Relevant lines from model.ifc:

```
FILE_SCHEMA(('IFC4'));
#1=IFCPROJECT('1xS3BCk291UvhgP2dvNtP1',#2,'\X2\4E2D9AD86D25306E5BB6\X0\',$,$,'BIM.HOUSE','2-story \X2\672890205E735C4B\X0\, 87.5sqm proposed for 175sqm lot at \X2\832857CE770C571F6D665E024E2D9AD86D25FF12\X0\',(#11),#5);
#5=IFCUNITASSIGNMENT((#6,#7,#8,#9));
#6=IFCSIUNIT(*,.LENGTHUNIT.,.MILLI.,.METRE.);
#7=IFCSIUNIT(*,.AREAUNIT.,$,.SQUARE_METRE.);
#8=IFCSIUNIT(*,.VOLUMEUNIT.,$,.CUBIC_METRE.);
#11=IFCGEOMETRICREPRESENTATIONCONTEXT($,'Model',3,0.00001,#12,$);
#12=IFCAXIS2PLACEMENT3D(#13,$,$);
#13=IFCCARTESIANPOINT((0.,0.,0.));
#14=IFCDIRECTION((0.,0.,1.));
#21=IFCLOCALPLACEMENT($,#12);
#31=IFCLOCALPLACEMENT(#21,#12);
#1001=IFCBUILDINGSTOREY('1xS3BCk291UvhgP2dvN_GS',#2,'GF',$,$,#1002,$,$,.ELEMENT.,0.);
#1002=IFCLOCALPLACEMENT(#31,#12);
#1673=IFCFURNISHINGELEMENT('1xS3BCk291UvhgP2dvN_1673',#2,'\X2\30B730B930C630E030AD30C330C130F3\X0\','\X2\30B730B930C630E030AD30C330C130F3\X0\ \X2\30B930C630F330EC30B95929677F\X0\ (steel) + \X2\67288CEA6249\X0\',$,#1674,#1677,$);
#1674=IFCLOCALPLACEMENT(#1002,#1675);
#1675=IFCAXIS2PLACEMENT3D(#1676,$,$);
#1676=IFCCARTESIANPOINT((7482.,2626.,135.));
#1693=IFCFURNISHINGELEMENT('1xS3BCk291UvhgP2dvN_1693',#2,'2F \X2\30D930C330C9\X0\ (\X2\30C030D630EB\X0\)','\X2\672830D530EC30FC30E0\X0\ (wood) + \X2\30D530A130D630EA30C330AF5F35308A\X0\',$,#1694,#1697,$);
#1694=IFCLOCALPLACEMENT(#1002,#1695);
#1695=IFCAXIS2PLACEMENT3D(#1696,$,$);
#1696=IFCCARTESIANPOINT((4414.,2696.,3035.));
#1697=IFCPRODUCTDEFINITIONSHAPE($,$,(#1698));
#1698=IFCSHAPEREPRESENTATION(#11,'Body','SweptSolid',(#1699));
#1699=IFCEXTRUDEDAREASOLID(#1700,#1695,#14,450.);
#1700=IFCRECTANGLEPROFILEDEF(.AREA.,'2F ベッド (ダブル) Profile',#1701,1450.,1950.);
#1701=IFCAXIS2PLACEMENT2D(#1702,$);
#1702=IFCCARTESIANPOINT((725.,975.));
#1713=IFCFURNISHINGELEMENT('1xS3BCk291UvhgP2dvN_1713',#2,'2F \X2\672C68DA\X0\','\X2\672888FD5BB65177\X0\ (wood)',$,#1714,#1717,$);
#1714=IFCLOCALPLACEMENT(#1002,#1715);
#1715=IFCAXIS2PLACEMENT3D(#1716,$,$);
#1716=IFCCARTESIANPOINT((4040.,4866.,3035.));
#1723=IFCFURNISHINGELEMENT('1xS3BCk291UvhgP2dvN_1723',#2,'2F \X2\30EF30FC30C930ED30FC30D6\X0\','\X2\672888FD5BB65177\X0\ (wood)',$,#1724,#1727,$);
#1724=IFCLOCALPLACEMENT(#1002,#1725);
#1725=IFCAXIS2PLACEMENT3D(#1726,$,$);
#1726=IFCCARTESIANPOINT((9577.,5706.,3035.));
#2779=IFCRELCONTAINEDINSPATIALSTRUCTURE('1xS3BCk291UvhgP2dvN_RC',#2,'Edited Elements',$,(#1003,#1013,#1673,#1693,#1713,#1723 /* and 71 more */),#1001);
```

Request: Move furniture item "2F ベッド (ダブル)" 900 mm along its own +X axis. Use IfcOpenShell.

```python
import ifcopenshell
import ifcopenshell.api.geometry
import ifcopenshell.util.placement

model = ifcopenshell.open("model.ifc")

item = model.by_id(1693)
matrix = ifcopenshell.util.placement.get_local_placement(item.ObjectPlacement)
matrix[:3, 3] += matrix[:3, 0] * 900.0
ifcopenshell.api.geometry.edit_object_placement(model, product=item, matrix=matrix, is_si=False)

print(ifcopenshell.util.placement.get_local_placement(item.ObjectPlacement).round(3) + 0.0)

model.write("model_rev.ifc")
```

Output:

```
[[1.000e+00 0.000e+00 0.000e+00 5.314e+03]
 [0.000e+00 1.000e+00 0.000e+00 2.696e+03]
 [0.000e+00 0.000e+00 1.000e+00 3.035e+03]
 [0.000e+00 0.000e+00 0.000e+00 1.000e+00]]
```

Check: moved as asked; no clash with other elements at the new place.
